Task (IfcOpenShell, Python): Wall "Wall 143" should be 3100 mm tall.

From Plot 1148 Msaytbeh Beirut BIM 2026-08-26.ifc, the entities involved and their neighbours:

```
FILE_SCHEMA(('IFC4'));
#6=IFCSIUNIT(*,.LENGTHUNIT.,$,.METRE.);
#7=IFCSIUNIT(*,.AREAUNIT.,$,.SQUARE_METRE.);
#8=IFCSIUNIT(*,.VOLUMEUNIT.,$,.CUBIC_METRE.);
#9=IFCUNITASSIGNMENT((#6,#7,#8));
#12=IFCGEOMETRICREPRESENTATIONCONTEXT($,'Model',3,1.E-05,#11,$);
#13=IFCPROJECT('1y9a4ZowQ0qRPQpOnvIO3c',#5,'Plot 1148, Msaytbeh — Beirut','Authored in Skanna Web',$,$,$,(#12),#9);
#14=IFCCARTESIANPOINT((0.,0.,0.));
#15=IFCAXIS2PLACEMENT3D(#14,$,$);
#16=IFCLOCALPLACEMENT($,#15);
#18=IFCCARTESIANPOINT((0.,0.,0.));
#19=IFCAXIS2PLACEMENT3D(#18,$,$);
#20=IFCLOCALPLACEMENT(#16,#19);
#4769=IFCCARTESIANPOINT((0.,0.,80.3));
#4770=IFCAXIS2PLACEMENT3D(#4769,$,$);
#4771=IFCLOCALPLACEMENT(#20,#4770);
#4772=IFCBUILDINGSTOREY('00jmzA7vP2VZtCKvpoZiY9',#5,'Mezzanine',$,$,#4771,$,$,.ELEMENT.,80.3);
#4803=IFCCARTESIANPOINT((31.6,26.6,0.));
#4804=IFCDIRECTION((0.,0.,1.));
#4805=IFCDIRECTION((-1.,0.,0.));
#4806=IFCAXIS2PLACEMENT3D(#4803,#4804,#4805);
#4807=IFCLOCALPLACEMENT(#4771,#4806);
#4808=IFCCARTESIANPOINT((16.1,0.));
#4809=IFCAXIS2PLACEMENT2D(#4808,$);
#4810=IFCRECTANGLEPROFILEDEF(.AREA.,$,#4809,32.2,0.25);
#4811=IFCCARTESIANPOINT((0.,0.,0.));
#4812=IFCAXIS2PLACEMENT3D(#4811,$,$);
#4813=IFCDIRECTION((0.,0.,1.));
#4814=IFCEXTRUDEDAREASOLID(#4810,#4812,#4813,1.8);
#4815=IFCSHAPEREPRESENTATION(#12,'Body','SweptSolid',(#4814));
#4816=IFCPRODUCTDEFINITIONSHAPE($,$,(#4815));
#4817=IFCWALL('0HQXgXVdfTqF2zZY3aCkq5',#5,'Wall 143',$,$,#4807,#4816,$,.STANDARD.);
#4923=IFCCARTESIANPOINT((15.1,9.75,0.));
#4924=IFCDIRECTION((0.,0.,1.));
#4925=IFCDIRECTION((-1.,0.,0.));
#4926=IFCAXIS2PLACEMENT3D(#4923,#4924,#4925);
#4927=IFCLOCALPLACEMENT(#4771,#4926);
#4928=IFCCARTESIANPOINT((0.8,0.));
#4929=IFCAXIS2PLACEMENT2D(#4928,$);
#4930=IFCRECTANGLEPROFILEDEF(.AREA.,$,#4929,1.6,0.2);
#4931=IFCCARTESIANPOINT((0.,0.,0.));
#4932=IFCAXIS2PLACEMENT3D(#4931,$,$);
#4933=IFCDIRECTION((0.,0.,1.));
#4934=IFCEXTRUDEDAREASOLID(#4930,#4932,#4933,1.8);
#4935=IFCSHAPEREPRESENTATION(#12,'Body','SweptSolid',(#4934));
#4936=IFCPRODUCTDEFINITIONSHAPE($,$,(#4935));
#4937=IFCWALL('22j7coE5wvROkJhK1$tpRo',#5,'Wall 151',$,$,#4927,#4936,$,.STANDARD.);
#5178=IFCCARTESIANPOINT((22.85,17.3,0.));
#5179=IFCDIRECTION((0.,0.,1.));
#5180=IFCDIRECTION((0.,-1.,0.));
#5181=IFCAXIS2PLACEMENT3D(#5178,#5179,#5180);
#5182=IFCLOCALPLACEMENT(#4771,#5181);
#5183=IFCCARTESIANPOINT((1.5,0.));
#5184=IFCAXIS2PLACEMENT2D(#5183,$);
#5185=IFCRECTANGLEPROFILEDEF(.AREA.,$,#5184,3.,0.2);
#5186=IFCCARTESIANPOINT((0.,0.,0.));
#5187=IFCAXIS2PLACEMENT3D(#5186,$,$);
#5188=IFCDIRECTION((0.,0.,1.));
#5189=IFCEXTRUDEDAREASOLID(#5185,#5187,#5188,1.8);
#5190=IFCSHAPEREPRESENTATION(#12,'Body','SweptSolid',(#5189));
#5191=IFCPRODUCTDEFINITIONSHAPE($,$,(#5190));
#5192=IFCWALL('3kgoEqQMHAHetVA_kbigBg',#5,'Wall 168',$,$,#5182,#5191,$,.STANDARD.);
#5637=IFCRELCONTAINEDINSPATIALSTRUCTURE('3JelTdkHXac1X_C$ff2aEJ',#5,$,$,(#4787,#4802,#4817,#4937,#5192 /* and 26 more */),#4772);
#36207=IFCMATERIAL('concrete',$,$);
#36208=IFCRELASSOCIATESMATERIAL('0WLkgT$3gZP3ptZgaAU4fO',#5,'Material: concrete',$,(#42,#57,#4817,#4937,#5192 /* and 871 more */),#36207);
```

```python
import ifcopenshell
import ifcopenshell.geom
import ifcopenshell.util.shape
import ifcopenshell.util.unit

model = ifcopenshell.open("Plot 1148 Msaytbeh Beirut BIM 2026-08-26.ifc")
unit_scale = ifcopenshell.util.unit.calculate_unit_scale(model)
settings = ifcopenshell.geom.settings()


def volume(element):
    """Net volume in cubic metres, openings subtracted."""
    shape = ifcopenshell.geom.create_shape(settings, element)
    return ifcopenshell.util.shape.get_volume(shape.geometry)


wall = model.by_guid("0HQXgXVdfTqF2zZY3aCkq5")
before = volume(wall)

body = next(r for r in wall.Representation.Representations if r.RepresentationIdentifier == "Body")
solid = body.Items[0]
old_height = solid.Depth
solid.Depth = 3.1 / unit_scale
after = volume(wall)

print(f"height {old_height:g} -> {solid.Depth:g}, volume {before:.3f} -> {after:.3f} m3")

model.write("Plot 1148 Msaytbeh Beirut BIM 2026-08-26-out.ifc")
```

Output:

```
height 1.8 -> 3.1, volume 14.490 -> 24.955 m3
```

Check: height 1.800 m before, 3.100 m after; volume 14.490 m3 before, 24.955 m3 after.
